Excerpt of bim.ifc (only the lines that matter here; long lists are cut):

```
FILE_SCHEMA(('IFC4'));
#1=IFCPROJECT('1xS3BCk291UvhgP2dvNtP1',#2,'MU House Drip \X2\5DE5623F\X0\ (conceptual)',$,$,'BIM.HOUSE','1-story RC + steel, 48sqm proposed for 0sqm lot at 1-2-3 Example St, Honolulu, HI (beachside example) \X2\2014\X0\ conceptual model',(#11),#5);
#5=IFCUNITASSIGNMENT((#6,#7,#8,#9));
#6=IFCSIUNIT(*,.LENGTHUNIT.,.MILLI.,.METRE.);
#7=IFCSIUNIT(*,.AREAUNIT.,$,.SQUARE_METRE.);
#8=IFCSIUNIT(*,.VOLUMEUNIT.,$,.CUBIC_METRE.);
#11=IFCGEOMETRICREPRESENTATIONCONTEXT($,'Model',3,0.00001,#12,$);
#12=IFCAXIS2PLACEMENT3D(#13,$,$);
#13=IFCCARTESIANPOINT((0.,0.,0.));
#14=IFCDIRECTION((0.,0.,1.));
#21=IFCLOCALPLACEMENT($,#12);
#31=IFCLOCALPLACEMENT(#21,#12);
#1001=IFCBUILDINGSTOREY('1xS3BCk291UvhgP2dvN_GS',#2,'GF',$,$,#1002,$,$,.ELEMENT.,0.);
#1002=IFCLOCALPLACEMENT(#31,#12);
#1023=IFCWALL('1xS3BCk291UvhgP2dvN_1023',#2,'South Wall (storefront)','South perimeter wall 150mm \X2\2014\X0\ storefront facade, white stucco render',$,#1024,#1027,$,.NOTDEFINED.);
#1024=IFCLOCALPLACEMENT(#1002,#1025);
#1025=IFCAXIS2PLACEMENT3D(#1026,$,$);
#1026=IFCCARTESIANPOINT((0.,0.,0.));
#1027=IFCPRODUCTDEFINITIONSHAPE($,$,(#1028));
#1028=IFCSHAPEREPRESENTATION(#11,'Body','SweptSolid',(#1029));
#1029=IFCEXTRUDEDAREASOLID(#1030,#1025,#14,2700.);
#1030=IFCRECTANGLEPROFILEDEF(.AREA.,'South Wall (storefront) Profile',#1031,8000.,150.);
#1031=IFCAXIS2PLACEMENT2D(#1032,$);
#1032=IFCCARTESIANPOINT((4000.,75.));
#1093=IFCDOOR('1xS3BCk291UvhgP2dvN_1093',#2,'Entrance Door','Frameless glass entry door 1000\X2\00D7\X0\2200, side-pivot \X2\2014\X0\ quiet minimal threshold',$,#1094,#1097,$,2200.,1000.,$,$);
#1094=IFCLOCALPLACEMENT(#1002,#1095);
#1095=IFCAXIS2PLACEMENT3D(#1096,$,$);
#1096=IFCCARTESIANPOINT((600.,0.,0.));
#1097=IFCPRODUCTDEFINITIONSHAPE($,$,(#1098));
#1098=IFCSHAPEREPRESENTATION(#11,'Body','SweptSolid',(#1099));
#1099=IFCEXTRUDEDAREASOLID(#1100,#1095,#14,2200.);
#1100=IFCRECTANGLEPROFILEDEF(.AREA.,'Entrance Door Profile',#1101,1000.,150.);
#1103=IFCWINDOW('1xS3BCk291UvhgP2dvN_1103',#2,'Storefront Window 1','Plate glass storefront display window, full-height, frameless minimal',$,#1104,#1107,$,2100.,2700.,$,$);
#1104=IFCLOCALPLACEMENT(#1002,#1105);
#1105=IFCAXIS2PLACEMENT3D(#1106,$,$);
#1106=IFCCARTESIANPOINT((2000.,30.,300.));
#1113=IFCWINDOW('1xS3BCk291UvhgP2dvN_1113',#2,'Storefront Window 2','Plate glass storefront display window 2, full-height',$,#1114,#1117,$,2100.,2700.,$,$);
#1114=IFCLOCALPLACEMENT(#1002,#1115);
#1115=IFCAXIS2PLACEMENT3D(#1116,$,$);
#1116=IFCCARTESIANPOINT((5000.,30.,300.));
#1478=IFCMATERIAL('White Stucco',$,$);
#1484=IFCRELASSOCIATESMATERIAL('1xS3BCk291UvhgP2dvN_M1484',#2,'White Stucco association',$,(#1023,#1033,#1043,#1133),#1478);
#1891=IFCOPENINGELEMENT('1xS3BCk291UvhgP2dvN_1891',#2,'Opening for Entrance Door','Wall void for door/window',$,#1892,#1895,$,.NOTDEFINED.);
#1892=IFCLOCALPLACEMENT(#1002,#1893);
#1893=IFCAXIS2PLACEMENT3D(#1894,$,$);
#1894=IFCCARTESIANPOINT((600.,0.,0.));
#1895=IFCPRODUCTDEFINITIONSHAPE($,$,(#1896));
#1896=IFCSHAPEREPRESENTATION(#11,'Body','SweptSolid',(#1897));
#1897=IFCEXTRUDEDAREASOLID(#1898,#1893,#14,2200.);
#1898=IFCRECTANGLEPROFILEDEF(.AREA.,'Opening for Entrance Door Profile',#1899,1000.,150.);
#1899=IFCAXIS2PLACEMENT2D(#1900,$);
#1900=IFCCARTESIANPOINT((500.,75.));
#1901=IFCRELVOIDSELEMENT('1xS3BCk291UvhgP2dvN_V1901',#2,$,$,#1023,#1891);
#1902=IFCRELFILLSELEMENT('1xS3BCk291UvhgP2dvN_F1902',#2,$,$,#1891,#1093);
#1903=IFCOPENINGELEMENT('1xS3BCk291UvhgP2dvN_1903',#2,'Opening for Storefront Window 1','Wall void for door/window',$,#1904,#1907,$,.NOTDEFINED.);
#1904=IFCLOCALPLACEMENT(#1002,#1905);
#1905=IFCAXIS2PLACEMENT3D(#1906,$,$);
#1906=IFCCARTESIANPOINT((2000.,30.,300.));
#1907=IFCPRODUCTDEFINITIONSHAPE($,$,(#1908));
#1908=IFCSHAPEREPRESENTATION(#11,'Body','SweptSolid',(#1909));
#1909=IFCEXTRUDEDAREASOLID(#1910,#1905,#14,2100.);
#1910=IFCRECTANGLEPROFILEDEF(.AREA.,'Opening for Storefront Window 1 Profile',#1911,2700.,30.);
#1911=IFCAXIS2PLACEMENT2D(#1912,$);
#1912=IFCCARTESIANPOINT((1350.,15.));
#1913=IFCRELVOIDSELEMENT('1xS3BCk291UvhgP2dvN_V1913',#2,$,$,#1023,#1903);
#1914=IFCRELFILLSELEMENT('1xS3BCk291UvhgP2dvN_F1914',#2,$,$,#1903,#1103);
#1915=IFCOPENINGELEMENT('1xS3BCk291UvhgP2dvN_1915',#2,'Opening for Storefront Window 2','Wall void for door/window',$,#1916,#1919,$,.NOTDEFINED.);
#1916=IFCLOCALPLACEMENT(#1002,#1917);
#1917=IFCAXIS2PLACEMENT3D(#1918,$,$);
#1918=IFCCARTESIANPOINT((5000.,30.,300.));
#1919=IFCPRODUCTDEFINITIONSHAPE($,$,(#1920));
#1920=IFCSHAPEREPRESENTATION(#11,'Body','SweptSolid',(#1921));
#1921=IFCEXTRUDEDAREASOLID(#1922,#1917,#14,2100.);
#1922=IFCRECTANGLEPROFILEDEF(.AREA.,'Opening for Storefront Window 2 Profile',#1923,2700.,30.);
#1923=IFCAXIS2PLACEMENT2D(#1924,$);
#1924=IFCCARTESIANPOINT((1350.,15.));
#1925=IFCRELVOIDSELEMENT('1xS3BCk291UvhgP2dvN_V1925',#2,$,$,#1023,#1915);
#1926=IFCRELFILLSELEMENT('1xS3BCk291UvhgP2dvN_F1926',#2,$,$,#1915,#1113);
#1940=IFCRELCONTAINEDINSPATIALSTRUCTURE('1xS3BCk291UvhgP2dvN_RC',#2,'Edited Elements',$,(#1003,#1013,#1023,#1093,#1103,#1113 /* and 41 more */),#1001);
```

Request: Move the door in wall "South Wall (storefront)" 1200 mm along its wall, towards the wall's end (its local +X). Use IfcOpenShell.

```python
import ifcopenshell
import ifcopenshell.api.geometry
import ifcopenshell.util.placement
import ifcopenshell.util.unit

model = ifcopenshell.open("bim.ifc")
unit_scale = ifcopenshell.util.unit.calculate_unit_scale(model)

door = model.by_guid("1xS3BCk291UvhgP2dvN_1093")
opening = door.FillsVoids[0].RelatingOpeningElement
wall = opening.VoidsElements[0].RelatingBuildingElement

wall_matrix = ifcopenshell.util.placement.get_local_placement(wall.ObjectPlacement)
shift = wall_matrix[:3, 0] * 1.2 / unit_scale
before = ifcopenshell.util.placement.get_local_placement(door.ObjectPlacement)[:3, 3].copy()

# The door is not placed relative to its opening, so move both.
for product in (opening, door):
    matrix = ifcopenshell.util.placement.get_local_placement(product.ObjectPlacement)
    matrix[:3, 3] += shift
    ifcopenshell.api.geometry.edit_object_placement(model, product=product, matrix=matrix, is_si=False)

after = ifcopenshell.util.placement.get_local_placement(door.ObjectPlacement)[:3, 3]
print("door moved by", (after - before).round(3) + 0.0)

model.write("bim_updated.ifc")
```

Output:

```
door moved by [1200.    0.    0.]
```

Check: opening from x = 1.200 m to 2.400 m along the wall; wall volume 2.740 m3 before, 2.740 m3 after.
